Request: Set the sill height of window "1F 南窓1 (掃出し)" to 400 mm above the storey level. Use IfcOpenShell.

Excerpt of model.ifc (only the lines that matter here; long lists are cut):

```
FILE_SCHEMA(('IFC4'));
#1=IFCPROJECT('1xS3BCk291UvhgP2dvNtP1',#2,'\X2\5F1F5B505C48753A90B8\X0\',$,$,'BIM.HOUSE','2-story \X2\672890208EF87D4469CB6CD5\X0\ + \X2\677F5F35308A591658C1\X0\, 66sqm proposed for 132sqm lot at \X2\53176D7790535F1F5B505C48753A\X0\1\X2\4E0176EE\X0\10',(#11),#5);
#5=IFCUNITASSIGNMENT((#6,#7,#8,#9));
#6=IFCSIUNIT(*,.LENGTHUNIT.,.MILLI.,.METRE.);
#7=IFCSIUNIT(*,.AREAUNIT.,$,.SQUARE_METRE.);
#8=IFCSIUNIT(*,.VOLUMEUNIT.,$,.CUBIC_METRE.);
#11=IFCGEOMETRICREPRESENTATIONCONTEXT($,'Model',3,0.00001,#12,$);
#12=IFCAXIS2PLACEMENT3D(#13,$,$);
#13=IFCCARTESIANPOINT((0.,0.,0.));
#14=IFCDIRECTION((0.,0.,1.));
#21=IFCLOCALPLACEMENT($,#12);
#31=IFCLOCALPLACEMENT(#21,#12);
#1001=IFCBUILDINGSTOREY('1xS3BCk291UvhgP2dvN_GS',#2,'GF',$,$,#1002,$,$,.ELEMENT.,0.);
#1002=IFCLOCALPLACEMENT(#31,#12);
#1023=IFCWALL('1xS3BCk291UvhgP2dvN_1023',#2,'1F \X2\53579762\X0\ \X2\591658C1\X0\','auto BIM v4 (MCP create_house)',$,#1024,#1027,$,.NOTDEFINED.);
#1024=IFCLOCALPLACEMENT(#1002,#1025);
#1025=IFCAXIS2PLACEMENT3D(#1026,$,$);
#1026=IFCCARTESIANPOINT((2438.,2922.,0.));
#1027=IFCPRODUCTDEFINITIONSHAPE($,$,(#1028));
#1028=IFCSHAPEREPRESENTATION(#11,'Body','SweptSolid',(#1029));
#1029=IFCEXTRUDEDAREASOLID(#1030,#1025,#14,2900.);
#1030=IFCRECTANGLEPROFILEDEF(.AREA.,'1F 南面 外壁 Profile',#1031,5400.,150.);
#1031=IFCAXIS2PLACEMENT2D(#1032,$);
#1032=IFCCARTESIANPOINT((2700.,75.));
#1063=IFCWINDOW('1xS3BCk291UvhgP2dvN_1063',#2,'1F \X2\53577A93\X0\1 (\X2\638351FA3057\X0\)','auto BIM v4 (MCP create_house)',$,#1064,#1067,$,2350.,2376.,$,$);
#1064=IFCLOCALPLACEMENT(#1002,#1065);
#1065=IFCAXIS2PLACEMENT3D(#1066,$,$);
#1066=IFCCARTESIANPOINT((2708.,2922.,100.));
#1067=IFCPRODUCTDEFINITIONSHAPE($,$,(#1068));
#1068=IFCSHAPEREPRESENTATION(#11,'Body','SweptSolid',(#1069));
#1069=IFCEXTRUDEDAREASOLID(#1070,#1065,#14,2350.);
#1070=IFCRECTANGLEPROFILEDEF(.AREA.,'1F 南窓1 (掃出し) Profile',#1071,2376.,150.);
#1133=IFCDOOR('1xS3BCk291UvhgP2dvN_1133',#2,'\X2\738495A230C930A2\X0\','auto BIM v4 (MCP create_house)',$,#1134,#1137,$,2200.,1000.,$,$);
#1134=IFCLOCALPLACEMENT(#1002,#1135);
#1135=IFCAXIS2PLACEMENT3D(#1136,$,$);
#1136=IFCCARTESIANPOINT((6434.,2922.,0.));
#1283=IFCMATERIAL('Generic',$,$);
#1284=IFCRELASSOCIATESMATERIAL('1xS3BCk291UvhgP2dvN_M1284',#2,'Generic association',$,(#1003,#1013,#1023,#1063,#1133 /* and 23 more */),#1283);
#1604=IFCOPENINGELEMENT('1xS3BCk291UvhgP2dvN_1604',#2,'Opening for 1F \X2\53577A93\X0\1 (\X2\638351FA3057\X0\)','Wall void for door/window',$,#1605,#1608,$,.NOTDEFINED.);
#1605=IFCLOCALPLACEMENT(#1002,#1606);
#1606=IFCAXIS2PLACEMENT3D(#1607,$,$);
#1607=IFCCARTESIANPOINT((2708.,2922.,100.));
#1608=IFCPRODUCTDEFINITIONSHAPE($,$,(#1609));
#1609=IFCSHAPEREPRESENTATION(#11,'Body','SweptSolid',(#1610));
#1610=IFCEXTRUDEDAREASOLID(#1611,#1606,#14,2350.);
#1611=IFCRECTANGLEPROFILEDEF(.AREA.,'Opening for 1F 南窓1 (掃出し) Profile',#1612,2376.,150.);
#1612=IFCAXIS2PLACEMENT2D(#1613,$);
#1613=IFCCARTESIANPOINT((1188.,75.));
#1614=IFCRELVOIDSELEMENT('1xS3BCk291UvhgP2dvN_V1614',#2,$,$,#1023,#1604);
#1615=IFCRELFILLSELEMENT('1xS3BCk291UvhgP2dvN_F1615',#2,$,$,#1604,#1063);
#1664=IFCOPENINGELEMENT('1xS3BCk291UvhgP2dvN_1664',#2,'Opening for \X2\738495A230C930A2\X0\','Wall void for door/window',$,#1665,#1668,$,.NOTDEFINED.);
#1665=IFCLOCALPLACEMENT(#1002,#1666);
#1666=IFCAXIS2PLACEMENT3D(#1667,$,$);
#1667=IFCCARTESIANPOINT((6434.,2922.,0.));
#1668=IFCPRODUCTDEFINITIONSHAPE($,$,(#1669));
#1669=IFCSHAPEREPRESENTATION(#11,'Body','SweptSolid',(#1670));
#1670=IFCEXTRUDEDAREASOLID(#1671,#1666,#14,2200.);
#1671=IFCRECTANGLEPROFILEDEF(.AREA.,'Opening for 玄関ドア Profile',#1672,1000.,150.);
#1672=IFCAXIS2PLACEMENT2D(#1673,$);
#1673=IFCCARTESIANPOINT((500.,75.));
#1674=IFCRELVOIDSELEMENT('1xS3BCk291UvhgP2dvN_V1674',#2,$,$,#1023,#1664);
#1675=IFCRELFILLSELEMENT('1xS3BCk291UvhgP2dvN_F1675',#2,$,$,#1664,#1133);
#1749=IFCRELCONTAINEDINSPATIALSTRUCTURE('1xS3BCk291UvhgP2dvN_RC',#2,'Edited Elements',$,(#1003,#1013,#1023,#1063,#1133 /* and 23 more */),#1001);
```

```python
import numpy as np
import ifcopenshell
import ifcopenshell.api.geometry
import ifcopenshell.geom
import ifcopenshell.util.element
import ifcopenshell.util.placement
import ifcopenshell.util.shape
import ifcopenshell.util.unit

model = ifcopenshell.open("model.ifc")
unit_scale = ifcopenshell.util.unit.calculate_unit_scale(model)

window = model.by_guid("1xS3BCk291UvhgP2dvN_1063")
opening = window.FillsVoids[0].RelatingOpeningElement
storey = ifcopenshell.util.element.get_container(window, ifc_class="IfcBuildingStorey")
level = ifcopenshell.util.placement.get_local_placement(storey.ObjectPlacement)[2, 3]

# The opening's origin need not be at the sill, so measure its lowest point.
shape = ifcopenshell.geom.create_shape(ifcopenshell.geom.settings(), opening)
bottom = ifcopenshell.util.shape.get_shape_bottom_elevation(shape, shape.geometry) / unit_scale
dz = level + 0.4 / unit_scale - bottom

shift = np.array([0.0, 0.0, dz])
# The window is not placed relative to its opening, so move both.
for product in (opening, window):
    matrix = ifcopenshell.util.placement.get_local_placement(product.ObjectPlacement)
    matrix[:3, 3] += shift
    ifcopenshell.api.geometry.edit_object_placement(model, product=product, matrix=matrix, is_si=False)

print(f"moved by {dz * unit_scale:+.3f} m")

model.write("model_rev.ifc")
```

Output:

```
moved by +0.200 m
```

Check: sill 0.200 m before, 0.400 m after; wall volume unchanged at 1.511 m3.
